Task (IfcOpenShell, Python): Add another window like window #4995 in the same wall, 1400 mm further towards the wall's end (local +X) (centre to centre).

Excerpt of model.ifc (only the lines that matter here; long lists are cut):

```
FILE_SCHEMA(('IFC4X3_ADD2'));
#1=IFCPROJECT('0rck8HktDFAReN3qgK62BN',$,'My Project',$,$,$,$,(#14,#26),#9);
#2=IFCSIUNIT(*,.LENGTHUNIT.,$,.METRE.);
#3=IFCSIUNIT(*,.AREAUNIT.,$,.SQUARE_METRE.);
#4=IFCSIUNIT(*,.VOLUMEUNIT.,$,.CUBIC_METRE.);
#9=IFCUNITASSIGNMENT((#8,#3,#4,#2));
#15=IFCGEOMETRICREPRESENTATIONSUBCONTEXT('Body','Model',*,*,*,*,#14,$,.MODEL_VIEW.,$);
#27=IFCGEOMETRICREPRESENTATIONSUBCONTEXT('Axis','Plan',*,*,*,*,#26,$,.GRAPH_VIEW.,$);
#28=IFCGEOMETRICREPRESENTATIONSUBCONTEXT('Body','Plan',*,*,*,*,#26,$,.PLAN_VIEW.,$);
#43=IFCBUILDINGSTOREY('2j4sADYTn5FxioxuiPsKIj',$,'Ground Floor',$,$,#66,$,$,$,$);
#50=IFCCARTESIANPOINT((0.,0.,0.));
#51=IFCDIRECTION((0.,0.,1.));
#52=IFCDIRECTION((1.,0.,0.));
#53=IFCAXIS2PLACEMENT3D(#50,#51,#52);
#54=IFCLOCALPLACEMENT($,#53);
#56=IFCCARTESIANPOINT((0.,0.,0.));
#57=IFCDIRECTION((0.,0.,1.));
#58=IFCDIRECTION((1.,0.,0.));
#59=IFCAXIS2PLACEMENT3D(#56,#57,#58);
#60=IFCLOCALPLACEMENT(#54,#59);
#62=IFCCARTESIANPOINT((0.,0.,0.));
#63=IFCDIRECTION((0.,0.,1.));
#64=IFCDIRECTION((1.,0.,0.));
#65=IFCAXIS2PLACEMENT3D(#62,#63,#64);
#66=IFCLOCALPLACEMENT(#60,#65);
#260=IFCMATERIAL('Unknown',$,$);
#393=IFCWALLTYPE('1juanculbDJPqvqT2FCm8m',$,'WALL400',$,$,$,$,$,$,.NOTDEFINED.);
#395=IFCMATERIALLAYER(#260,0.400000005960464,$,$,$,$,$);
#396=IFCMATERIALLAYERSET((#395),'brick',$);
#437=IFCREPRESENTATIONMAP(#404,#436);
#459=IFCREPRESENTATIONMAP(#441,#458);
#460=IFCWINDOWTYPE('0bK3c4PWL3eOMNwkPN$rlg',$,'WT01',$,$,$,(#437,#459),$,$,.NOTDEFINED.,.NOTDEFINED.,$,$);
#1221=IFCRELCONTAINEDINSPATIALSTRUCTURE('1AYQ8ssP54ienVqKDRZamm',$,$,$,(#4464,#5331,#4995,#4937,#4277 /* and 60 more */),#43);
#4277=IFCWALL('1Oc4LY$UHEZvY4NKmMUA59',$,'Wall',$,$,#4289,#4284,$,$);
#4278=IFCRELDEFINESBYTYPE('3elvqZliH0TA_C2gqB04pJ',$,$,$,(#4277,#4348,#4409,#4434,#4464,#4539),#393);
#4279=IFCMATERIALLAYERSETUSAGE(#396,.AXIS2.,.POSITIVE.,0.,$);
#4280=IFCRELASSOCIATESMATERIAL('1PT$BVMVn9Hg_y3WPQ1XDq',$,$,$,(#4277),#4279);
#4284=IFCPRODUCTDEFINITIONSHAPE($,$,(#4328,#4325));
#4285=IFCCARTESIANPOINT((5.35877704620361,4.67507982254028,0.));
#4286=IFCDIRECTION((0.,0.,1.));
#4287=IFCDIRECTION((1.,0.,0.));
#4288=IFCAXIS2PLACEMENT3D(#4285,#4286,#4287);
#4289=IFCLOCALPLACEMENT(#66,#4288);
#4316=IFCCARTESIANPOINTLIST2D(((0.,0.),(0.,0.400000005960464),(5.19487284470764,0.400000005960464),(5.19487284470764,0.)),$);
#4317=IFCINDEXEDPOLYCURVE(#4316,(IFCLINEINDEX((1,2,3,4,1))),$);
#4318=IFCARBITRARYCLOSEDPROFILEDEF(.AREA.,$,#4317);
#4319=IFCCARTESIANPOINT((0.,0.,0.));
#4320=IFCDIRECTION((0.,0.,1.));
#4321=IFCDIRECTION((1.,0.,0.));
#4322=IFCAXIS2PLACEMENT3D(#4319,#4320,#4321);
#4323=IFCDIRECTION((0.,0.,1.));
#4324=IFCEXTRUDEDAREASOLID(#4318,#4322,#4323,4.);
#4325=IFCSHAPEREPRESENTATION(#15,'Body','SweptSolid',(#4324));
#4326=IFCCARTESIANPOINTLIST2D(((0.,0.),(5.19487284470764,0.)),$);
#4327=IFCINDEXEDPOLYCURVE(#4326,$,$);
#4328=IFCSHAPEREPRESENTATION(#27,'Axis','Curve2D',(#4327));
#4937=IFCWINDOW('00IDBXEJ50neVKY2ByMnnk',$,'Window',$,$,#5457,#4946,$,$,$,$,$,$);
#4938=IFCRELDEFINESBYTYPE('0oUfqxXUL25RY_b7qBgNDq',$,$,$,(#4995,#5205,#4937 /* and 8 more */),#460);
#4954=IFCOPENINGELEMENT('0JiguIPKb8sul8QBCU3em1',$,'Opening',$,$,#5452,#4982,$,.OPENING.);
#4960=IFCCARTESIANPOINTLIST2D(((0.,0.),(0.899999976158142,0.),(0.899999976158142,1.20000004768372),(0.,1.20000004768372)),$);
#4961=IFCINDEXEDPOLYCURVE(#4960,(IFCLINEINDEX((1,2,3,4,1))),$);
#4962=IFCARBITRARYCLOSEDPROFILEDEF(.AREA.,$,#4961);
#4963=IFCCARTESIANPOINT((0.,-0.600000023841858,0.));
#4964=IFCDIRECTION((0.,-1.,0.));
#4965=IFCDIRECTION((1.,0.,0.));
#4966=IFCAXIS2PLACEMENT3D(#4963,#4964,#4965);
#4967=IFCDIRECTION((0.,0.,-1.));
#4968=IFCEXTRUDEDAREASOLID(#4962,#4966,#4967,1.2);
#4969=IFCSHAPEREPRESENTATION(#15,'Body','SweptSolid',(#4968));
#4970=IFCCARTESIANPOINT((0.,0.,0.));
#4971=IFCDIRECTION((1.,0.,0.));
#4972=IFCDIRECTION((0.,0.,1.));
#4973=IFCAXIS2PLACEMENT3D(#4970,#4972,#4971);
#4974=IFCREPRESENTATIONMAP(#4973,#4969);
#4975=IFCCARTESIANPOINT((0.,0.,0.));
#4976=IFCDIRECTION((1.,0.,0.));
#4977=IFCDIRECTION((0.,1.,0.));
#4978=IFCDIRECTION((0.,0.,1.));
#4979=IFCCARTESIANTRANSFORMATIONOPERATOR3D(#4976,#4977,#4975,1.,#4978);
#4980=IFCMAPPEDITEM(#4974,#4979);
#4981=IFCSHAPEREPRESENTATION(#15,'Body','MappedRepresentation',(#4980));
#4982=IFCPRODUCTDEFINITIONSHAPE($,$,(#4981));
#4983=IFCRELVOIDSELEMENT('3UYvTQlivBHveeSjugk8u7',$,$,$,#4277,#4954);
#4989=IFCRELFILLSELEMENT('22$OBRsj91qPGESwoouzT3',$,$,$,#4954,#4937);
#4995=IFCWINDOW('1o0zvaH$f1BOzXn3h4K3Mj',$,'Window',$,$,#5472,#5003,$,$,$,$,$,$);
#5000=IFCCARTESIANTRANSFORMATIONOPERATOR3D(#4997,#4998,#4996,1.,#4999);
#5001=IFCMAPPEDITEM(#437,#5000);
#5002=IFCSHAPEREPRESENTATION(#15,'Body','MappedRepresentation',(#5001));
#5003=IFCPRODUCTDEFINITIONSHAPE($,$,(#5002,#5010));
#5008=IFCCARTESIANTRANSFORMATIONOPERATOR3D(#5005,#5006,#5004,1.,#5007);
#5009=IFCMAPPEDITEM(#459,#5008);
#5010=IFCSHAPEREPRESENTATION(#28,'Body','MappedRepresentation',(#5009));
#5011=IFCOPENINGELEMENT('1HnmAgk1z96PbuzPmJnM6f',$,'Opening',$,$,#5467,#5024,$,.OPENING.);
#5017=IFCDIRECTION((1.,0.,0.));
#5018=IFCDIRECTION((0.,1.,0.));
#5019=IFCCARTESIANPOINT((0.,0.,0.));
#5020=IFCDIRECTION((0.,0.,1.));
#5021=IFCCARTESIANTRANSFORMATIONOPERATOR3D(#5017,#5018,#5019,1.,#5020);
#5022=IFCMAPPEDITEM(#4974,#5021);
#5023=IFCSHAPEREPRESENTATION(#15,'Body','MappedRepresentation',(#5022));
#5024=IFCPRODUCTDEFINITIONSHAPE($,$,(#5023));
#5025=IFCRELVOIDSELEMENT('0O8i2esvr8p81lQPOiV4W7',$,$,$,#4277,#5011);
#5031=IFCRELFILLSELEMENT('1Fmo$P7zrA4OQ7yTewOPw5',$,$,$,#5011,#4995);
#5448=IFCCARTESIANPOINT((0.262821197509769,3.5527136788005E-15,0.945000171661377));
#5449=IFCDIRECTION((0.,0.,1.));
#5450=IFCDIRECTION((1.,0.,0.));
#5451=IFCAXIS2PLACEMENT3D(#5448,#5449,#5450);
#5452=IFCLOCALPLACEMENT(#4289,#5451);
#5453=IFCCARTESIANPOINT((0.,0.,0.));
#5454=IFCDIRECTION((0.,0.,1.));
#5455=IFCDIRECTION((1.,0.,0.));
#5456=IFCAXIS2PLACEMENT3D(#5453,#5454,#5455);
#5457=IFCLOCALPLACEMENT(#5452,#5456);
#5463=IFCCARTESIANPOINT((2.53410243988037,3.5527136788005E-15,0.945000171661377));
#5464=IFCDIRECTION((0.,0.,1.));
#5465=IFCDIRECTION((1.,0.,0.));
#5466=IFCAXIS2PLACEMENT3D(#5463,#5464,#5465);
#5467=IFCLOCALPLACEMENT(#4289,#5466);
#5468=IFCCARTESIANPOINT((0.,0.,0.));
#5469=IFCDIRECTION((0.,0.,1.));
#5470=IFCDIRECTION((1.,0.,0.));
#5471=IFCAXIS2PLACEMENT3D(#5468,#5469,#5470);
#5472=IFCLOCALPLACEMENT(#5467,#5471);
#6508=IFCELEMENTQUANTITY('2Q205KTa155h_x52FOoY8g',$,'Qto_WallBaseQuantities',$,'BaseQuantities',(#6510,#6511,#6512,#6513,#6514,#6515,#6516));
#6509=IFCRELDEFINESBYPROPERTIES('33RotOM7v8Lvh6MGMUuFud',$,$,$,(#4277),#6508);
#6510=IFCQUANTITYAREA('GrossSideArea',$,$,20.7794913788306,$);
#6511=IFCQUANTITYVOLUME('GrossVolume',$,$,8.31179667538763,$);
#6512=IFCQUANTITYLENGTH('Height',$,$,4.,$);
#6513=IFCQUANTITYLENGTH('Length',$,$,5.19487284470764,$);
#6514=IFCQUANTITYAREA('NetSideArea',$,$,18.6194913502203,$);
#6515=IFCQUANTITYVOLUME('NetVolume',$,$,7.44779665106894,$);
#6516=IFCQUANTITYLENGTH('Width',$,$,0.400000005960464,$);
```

```python
import ifcopenshell
import ifcopenshell.api.feature
import ifcopenshell.api.geometry
import ifcopenshell.api.pset
import ifcopenshell.api.root
import ifcopenshell.geom
import ifcopenshell.util.element
import ifcopenshell.util.placement
import ifcopenshell.util.shape
import ifcopenshell.util.unit

model = ifcopenshell.open("model.ifc")
area_scale = ifcopenshell.util.unit.calculate_unit_scale(model, "AREAUNIT")
volume_scale = ifcopenshell.util.unit.calculate_unit_scale(model, "VOLUMEUNIT")
settings = ifcopenshell.geom.settings()


def volume(element):
    """Net volume in cubic metres, openings subtracted."""
    shape = ifcopenshell.geom.create_shape(settings, element)
    return ifcopenshell.util.shape.get_volume(shape.geometry)


window = model.by_id(4995)
opening = window.FillsVoids[0].RelatingOpeningElement
wall = opening.VoidsElements[0].RelatingBuildingElement
before = volume(wall)
shift = ifcopenshell.util.placement.get_local_placement(wall.ObjectPlacement)[:3, 0] * 1.4

# copy_class copies the void relationship, type, container and properties, but no geometry.
new_opening = ifcopenshell.api.root.copy_class(model, product=opening)
new_opening.Representation = ifcopenshell.util.element.copy_deep(
    model, opening.Representation, exclude=["IfcGeometricRepresentationContext", "IfcRepresentationMap"]
)
new_window = ifcopenshell.api.root.copy_class(model, product=window)
new_window.Representation = ifcopenshell.util.element.copy_deep(
    model, window.Representation, exclude=["IfcGeometricRepresentationContext", "IfcRepresentationMap"]
)
ifcopenshell.api.feature.add_filling(model, opening=new_opening, element=new_window)

for old, new in ((opening, new_opening), (window, new_window)):
    matrix = ifcopenshell.util.placement.get_local_placement(old.ObjectPlacement)
    matrix[:3, 3] += shift
    ifcopenshell.api.geometry.edit_object_placement(model, product=new, matrix=matrix, is_si=False)

after = volume(wall)
thickness = 0.4  # wall thickness in metres

# Update the wall's stored quantities.
qto = model.by_id(ifcopenshell.util.element.get_pset(wall, "Qto_WallBaseQuantities", should_inherit=False)["id"])
ifcopenshell.api.pset.edit_qto(model, qto=qto, properties={
    "NetSideArea": after / thickness / area_scale,
    "NetVolume": after / volume_scale,
})

print(f"wall volume {before:.3f} -> {after:.3f} m3")

model.write("model_v2.ifc")
```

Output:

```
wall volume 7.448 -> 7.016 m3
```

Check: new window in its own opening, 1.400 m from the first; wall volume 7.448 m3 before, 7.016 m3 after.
